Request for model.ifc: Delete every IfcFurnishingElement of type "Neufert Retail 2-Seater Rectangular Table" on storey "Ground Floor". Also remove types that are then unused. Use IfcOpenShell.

First a look at what the model holds.

```python
import ifcopenshell
import ifcopenshell.util.element

model = ifcopenshell.open("model.ifc")
print(model.schema)
storey = next(s for s in model.by_type("IfcBuildingStorey") if s.Name == "Ground Floor")
furniture = [e for e in ifcopenshell.util.element.get_decomposition(storey) if e.is_a("IfcFurnishingElement")]
seen = {}
for e in furniture:
    element_type = ifcopenshell.util.element.get_type(e)
    name = element_type.Name if element_type not in (None, e) else None
    seen[name] = seen.get(name, 0) + 1
for name, count in sorted(seen.items(), key=str):
    print(count, "x", name)
```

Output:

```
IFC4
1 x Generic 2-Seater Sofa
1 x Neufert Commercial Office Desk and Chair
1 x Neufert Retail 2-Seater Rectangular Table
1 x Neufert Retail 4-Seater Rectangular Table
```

```python
import ifcopenshell
import ifcopenshell.api.root
import ifcopenshell.util.element

model = ifcopenshell.open("model.ifc")

storey = next(s for s in model.by_type("IfcBuildingStorey") if s.Name == "Ground Floor")
furniture = [e for e in ifcopenshell.util.element.get_decomposition(storey) if e.is_a("IfcFurnishingElement")]
targets = [e for e in furniture if (t := ifcopenshell.util.element.get_type(e)) not in (None, e) and t.Name == "Neufert Retail 2-Seater Rectangular Table"]
types = {ifcopenshell.util.element.get_type(e) for e in targets} - {None, *targets}

for e in targets:
    ifcopenshell.api.root.remove_product(model, product=e)
print(len(targets), "removed")

unused = [t for t in types if not ifcopenshell.util.element.get_types(t)]
for t in unused:
    ifcopenshell.api.root.remove_product(model, product=t)
print(len(unused), "unused types removed")

model.write("model-out.ifc")
```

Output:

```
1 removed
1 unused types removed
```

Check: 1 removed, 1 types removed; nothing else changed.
